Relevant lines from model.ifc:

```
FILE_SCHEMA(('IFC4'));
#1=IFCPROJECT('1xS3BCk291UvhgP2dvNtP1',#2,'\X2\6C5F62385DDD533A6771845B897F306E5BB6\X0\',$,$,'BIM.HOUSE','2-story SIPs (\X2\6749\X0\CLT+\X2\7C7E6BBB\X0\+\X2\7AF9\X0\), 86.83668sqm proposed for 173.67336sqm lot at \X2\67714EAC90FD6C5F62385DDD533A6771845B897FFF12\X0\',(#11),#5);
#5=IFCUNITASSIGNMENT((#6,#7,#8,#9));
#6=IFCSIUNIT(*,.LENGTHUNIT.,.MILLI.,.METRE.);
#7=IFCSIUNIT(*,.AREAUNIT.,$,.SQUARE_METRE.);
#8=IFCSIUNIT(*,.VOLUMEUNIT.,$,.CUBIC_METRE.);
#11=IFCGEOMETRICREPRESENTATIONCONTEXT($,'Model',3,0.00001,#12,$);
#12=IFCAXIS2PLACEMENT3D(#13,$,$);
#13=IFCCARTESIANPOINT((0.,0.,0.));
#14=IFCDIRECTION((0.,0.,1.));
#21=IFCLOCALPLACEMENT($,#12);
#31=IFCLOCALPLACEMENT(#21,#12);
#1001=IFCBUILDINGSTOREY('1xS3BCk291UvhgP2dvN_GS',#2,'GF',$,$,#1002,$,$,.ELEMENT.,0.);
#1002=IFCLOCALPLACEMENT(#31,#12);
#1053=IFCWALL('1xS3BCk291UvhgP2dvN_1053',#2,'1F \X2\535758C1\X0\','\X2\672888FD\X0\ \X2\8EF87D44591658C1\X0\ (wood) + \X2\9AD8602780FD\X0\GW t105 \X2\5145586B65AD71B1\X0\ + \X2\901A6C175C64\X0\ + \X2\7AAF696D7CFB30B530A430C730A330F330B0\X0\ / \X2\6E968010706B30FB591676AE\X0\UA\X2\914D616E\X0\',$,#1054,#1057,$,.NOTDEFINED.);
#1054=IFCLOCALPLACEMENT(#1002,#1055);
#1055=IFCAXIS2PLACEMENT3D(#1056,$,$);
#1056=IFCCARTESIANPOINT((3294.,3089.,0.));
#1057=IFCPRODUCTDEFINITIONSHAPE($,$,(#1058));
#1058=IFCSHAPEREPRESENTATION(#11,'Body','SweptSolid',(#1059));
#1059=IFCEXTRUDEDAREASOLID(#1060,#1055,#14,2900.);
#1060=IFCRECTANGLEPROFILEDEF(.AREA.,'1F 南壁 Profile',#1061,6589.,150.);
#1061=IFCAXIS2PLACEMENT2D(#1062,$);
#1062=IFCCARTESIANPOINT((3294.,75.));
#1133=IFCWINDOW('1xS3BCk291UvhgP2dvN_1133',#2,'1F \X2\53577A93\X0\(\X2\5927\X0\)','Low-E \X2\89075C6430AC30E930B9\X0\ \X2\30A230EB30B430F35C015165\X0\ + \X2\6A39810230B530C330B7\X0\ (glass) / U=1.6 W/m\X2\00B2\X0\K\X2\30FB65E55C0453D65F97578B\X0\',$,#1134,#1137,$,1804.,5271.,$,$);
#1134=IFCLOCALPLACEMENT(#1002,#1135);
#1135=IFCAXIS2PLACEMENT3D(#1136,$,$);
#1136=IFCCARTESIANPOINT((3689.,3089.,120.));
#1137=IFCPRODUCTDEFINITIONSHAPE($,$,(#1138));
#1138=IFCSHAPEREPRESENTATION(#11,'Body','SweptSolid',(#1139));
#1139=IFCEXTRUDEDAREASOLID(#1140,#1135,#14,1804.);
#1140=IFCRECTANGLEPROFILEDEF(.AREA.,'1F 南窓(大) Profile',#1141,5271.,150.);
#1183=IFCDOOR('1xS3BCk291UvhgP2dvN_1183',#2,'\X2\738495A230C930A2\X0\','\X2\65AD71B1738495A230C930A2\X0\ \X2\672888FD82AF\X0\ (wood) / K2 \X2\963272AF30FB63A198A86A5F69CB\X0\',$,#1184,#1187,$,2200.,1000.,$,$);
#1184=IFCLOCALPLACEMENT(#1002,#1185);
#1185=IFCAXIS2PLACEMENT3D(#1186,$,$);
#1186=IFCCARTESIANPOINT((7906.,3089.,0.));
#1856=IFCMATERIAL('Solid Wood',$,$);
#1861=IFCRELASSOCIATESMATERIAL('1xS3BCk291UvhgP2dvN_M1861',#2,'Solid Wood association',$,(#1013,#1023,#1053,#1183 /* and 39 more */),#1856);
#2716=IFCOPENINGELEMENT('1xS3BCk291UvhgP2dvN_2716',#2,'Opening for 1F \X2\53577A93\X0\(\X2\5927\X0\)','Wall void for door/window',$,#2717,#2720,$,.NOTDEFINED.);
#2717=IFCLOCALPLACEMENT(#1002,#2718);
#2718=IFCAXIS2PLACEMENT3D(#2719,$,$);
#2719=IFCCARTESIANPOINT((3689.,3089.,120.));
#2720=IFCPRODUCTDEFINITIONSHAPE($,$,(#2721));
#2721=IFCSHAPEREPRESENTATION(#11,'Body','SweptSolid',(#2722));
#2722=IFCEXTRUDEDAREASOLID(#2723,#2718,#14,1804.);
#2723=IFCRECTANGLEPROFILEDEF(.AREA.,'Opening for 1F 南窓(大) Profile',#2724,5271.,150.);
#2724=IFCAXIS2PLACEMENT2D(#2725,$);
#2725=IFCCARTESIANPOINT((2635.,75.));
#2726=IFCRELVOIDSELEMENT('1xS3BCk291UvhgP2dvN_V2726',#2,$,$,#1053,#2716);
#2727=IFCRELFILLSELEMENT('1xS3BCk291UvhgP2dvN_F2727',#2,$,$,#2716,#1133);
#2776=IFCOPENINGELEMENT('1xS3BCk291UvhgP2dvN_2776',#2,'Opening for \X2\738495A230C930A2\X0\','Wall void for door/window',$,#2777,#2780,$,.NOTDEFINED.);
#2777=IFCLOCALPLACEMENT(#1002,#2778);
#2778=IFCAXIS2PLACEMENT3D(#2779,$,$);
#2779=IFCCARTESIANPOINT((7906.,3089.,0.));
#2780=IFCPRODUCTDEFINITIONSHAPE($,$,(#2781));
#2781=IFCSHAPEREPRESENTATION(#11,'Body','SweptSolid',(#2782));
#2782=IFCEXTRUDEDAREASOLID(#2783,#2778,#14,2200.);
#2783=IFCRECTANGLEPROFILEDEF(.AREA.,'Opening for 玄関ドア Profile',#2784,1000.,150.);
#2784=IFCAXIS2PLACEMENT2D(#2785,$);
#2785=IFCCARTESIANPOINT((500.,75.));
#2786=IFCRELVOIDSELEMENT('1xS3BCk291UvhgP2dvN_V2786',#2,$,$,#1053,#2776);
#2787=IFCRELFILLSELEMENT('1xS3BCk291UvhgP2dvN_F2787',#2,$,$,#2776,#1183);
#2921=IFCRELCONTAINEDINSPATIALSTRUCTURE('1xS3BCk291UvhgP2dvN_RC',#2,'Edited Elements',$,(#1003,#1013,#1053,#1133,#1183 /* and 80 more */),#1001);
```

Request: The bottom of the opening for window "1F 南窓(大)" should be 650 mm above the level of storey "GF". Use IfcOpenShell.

```python
import numpy as np
import ifcopenshell
import ifcopenshell.api.geometry
import ifcopenshell.geom
import ifcopenshell.util.element
import ifcopenshell.util.placement
import ifcopenshell.util.shape
import ifcopenshell.util.unit

model = ifcopenshell.open("model.ifc")
unit_scale = ifcopenshell.util.unit.calculate_unit_scale(model)

window = model.by_guid("1xS3BCk291UvhgP2dvN_1133")
opening = window.FillsVoids[0].RelatingOpeningElement
storey = ifcopenshell.util.element.get_container(window, ifc_class="IfcBuildingStorey")
level = ifcopenshell.util.placement.get_local_placement(storey.ObjectPlacement)[2, 3]

# The opening's origin need not be at the sill, so measure its lowest point.
shape = ifcopenshell.geom.create_shape(ifcopenshell.geom.settings(), opening)
bottom = ifcopenshell.util.shape.get_shape_bottom_elevation(shape, shape.geometry) / unit_scale
dz = level + 0.65 / unit_scale - bottom

shift = np.array([0.0, 0.0, dz])
# The window is not placed relative to its opening, so move both.
for product in (opening, window):
    matrix = ifcopenshell.util.placement.get_local_placement(product.ObjectPlacement)
    matrix[:3, 3] += shift
    ifcopenshell.api.geometry.edit_object_placement(model, product=product, matrix=matrix, is_si=False)

print(f"moved by {dz * unit_scale:+.3f} m")

model.write("model_rev.ifc")
```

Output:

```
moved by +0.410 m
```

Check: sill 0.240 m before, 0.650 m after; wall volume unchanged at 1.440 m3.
